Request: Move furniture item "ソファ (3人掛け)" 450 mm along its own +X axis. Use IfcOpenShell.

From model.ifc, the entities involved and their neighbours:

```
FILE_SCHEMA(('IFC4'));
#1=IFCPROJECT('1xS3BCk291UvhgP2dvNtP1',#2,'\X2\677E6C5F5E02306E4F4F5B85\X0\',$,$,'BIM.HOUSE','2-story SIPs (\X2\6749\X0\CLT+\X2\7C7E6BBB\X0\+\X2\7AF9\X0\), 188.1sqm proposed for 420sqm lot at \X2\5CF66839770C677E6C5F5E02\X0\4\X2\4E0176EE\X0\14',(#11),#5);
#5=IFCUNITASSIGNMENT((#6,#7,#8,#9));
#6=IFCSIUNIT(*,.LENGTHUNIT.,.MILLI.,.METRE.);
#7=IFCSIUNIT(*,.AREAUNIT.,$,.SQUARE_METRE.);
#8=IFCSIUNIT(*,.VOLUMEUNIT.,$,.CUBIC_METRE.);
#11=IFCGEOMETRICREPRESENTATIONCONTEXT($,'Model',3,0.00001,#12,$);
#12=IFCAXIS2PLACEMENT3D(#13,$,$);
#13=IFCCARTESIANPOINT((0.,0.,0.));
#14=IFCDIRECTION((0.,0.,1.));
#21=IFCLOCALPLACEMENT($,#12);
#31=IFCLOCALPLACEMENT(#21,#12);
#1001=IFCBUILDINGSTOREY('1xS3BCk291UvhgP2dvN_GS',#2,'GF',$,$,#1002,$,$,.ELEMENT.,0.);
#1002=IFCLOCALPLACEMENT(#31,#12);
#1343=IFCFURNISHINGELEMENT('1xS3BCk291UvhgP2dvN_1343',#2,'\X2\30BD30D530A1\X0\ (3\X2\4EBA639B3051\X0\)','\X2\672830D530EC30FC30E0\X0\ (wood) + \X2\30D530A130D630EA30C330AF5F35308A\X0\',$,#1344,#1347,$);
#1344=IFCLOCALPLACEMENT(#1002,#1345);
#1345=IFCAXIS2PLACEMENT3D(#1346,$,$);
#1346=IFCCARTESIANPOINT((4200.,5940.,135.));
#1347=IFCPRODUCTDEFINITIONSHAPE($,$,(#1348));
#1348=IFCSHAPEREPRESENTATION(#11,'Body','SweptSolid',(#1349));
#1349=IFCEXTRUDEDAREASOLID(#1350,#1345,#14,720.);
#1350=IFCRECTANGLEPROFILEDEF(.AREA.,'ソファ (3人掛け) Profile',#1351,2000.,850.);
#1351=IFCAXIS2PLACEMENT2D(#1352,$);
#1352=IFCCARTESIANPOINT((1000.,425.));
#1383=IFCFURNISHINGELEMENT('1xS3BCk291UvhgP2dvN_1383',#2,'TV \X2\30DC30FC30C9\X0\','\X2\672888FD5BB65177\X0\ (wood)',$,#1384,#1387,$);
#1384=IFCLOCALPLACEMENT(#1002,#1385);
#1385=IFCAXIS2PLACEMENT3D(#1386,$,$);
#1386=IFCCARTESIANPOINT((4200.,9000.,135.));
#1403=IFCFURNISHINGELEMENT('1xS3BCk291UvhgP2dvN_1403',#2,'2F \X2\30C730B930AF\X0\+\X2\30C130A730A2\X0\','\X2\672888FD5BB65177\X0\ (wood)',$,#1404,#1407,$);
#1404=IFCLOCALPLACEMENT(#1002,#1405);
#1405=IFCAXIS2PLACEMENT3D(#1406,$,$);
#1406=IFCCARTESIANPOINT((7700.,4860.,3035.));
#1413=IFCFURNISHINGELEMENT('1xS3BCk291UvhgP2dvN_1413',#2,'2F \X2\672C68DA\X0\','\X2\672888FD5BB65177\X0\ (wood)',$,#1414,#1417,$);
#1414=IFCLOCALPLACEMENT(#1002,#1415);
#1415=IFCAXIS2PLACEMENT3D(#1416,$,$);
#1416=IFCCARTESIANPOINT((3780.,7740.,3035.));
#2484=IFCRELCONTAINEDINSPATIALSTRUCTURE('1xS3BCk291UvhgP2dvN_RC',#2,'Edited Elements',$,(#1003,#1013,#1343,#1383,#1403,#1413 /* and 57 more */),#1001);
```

```python
import ifcopenshell
import ifcopenshell.api.geometry
import ifcopenshell.util.placement
import ifcopenshell.util.unit

model = ifcopenshell.open("model.ifc")
unit_scale = ifcopenshell.util.unit.calculate_unit_scale(model)

item = model.by_guid("1xS3BCk291UvhgP2dvN_1343")
matrix = ifcopenshell.util.placement.get_local_placement(item.ObjectPlacement)
matrix[:3, 3] += matrix[:3, 0] * 0.45 / unit_scale
ifcopenshell.api.geometry.edit_object_placement(model, product=item, matrix=matrix, is_si=False)

print(ifcopenshell.util.placement.get_local_placement(item.ObjectPlacement).round(3) + 0.0)

model.write("model_rev.ifc")
```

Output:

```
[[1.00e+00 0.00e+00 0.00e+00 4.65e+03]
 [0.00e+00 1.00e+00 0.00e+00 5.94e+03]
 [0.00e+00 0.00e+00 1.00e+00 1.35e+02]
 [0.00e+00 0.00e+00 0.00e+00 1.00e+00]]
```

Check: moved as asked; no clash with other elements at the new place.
